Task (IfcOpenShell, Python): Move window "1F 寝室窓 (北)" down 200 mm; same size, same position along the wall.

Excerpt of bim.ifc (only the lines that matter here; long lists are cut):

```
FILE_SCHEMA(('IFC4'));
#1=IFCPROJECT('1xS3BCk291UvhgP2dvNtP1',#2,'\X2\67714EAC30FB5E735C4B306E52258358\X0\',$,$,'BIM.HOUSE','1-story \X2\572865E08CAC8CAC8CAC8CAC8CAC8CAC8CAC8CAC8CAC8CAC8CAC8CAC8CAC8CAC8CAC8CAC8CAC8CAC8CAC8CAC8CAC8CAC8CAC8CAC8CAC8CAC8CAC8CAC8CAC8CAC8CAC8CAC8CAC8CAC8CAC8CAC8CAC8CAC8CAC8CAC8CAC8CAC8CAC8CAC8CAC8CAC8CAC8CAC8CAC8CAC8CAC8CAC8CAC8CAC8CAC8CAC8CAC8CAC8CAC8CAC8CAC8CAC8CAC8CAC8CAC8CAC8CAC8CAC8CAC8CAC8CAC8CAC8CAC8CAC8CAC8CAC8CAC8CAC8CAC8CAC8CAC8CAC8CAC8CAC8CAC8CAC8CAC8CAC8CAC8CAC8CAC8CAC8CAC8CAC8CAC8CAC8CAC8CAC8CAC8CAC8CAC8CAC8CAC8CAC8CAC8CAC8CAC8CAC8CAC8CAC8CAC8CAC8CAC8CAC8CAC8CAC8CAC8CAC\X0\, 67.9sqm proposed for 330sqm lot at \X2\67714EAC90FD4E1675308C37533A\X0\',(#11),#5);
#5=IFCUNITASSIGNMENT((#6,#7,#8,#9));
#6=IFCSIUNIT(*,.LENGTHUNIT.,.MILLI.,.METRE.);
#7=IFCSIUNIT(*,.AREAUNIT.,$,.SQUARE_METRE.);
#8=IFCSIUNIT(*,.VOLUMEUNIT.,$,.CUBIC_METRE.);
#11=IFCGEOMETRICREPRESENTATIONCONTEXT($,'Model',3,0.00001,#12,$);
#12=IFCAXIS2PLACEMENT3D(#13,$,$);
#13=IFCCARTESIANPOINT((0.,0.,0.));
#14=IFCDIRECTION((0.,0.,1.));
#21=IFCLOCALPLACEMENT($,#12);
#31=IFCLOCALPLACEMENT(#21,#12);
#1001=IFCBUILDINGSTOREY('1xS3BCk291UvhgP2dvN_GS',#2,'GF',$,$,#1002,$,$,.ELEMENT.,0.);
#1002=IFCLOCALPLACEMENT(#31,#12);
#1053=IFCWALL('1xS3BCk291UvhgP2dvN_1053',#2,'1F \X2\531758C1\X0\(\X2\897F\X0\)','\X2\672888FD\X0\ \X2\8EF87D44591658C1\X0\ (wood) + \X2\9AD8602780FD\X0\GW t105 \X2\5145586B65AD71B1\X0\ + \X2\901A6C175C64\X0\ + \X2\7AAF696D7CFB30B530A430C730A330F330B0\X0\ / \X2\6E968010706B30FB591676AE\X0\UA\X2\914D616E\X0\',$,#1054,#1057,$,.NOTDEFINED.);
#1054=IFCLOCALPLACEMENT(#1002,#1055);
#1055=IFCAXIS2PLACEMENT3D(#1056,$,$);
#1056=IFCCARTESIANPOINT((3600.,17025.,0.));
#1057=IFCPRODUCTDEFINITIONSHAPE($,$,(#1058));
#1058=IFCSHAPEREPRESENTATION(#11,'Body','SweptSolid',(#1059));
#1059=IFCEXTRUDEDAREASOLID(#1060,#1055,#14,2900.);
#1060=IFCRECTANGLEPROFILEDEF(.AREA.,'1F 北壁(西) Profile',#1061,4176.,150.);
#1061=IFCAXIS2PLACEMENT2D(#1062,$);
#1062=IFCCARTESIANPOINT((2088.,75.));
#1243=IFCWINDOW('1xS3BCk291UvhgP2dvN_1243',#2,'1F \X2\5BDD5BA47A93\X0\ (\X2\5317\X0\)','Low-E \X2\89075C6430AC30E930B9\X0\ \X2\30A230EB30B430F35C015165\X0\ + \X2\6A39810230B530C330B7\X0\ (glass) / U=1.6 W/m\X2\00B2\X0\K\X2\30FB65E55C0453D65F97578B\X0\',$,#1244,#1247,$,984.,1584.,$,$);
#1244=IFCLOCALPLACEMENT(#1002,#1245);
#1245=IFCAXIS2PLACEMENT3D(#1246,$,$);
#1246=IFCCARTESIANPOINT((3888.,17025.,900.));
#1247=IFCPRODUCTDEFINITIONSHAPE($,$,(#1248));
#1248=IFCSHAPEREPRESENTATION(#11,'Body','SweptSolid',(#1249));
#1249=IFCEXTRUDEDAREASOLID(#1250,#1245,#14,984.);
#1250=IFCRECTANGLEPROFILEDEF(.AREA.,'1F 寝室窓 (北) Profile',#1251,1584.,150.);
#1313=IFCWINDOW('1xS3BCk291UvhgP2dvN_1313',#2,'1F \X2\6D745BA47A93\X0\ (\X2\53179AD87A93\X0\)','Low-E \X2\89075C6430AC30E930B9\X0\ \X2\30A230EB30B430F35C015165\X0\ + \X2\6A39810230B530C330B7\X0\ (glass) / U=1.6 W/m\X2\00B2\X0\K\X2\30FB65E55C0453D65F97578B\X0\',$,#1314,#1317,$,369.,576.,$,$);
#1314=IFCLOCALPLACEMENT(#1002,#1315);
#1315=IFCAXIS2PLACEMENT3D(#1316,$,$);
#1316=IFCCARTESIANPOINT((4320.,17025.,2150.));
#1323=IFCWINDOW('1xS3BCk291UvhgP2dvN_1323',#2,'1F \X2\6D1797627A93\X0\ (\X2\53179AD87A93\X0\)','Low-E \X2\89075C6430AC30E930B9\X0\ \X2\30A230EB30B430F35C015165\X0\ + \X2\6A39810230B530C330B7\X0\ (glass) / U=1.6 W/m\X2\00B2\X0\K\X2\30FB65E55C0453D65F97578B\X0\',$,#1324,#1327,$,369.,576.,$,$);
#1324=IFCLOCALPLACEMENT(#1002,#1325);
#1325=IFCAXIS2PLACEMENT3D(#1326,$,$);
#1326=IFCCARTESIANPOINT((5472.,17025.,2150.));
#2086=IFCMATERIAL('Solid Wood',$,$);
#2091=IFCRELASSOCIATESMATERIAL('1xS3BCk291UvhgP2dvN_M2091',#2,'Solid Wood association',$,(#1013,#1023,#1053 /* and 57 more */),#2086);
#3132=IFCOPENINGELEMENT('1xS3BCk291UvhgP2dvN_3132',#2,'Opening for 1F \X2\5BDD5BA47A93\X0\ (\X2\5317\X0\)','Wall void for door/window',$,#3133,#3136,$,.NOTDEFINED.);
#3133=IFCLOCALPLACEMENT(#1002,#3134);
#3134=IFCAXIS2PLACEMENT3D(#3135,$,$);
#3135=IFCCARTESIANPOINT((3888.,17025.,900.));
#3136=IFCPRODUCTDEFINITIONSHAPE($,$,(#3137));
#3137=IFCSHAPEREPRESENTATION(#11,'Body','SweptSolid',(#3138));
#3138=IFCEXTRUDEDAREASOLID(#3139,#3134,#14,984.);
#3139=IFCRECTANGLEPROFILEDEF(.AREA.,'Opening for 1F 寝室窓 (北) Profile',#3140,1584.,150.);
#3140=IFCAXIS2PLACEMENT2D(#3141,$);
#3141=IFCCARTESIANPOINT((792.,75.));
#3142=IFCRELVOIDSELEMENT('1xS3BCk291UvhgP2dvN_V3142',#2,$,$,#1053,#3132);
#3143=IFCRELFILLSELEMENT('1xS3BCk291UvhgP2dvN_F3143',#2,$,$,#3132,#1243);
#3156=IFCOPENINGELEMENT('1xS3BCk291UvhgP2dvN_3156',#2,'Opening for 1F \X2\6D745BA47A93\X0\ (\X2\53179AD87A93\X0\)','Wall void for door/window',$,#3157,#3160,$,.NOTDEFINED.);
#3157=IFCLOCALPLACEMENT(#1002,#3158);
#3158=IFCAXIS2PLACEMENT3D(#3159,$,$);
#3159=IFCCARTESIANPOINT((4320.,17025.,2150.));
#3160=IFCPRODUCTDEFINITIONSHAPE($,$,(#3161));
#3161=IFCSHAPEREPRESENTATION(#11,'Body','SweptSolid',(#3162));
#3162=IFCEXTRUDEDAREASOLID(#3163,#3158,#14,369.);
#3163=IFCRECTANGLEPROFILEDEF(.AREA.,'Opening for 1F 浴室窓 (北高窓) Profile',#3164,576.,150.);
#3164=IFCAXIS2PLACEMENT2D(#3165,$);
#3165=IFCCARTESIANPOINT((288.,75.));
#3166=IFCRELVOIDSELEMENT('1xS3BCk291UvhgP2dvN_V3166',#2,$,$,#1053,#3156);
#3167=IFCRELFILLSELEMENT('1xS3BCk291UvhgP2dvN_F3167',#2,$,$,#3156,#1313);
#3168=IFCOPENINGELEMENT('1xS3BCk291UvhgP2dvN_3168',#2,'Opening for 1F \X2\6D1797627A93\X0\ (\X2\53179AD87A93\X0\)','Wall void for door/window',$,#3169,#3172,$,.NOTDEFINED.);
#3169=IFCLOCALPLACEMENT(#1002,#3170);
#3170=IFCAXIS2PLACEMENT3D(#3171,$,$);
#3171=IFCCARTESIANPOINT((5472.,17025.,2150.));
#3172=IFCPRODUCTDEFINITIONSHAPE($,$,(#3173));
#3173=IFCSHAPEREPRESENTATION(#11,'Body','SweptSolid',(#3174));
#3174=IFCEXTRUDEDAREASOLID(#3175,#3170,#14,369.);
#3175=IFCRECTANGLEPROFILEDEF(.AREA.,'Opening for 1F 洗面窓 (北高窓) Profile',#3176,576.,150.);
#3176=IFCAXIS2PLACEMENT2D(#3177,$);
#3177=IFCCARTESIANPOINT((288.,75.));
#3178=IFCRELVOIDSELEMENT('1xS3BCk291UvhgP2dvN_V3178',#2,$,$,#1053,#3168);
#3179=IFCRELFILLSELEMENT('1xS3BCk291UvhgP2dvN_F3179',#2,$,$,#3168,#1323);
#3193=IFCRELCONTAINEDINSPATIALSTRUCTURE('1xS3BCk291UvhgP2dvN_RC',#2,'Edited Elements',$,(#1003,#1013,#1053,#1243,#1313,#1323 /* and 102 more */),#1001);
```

```python
import numpy as np
import ifcopenshell
import ifcopenshell.api.geometry
import ifcopenshell.util.placement
import ifcopenshell.util.unit

model = ifcopenshell.open("bim.ifc")
unit_scale = ifcopenshell.util.unit.calculate_unit_scale(model)

window = model.by_guid("1xS3BCk291UvhgP2dvN_1243")
opening = window.FillsVoids[0].RelatingOpeningElement
dz = -200.0

shift = np.array([0.0, 0.0, dz])
# The window is not placed relative to its opening, so move both.
for product in (opening, window):
    matrix = ifcopenshell.util.placement.get_local_placement(product.ObjectPlacement)
    matrix[:3, 3] += shift
    ifcopenshell.api.geometry.edit_object_placement(model, product=product, matrix=matrix, is_si=False)

print(f"moved by {dz * unit_scale:+.3f} m")

model.write("bim_updated.ifc")
```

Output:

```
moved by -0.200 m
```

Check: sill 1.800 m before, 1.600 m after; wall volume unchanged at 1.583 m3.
